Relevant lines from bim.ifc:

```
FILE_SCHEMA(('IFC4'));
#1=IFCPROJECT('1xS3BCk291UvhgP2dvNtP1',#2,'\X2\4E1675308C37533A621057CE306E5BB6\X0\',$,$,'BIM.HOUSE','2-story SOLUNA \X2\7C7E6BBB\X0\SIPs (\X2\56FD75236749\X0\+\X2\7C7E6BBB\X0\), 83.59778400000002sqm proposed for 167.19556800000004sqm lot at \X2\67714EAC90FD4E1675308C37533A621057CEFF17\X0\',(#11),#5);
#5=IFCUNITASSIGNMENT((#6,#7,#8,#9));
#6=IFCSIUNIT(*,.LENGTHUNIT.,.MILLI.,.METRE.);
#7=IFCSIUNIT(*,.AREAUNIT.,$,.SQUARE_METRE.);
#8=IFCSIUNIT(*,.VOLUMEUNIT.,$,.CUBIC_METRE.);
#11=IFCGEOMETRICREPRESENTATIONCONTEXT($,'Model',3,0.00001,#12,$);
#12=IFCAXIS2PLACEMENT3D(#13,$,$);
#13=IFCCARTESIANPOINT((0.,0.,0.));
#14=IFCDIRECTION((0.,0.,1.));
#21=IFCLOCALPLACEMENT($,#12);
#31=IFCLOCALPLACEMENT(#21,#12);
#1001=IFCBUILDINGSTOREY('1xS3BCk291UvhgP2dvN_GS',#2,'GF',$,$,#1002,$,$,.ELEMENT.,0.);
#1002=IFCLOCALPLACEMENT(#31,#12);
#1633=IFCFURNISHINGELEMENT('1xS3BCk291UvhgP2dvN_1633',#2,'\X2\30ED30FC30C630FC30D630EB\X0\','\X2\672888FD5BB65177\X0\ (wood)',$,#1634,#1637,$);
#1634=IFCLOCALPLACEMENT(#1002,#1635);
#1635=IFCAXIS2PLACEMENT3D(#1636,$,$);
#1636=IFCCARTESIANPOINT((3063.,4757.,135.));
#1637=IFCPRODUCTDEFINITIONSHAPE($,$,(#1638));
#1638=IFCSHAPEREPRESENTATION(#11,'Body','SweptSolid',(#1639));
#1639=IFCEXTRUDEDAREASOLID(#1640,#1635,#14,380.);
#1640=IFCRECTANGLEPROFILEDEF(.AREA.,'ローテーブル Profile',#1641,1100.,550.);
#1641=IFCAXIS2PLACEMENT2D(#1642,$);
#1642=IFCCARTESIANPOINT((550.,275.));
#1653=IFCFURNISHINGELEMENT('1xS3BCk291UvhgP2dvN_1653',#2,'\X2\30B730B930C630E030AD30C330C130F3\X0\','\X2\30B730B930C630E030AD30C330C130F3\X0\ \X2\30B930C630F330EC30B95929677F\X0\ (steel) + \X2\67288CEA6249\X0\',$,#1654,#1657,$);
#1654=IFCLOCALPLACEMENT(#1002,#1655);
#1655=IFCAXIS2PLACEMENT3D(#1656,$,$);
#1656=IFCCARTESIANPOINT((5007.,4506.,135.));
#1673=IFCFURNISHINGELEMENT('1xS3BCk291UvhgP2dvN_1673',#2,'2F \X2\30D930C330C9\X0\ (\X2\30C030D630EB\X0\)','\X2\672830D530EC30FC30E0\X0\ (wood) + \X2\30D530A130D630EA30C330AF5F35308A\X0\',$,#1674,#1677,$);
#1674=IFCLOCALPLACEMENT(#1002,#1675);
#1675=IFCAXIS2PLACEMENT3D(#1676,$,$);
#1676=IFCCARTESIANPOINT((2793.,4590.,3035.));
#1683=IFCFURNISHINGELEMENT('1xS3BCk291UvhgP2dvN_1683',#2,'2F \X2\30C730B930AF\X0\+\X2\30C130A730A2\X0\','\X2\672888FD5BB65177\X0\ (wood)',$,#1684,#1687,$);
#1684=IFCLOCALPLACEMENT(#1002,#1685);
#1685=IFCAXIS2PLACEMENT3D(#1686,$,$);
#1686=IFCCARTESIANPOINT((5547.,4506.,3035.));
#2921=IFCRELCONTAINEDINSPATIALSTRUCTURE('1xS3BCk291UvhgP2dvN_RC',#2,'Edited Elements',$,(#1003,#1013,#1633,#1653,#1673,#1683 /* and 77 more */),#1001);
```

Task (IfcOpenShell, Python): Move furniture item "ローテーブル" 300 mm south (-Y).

```python
import ifcopenshell
import ifcopenshell.api.geometry
import ifcopenshell.util.placement
import ifcopenshell.util.unit

model = ifcopenshell.open("bim.ifc")
unit_scale = ifcopenshell.util.unit.calculate_unit_scale(model)

item = model.by_guid("1xS3BCk291UvhgP2dvN_1633")
matrix = ifcopenshell.util.placement.get_local_placement(item.ObjectPlacement)
matrix[1, 3] -= 0.3 / unit_scale
ifcopenshell.api.geometry.edit_object_placement(model, product=item, matrix=matrix, is_si=False)

print(ifcopenshell.util.placement.get_local_placement(item.ObjectPlacement).round(3) + 0.0)

model.write("bim_edited.ifc")
```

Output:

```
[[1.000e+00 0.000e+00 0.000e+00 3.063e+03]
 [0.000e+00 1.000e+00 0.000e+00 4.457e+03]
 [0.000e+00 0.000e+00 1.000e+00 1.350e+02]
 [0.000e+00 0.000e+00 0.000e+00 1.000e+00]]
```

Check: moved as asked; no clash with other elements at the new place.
